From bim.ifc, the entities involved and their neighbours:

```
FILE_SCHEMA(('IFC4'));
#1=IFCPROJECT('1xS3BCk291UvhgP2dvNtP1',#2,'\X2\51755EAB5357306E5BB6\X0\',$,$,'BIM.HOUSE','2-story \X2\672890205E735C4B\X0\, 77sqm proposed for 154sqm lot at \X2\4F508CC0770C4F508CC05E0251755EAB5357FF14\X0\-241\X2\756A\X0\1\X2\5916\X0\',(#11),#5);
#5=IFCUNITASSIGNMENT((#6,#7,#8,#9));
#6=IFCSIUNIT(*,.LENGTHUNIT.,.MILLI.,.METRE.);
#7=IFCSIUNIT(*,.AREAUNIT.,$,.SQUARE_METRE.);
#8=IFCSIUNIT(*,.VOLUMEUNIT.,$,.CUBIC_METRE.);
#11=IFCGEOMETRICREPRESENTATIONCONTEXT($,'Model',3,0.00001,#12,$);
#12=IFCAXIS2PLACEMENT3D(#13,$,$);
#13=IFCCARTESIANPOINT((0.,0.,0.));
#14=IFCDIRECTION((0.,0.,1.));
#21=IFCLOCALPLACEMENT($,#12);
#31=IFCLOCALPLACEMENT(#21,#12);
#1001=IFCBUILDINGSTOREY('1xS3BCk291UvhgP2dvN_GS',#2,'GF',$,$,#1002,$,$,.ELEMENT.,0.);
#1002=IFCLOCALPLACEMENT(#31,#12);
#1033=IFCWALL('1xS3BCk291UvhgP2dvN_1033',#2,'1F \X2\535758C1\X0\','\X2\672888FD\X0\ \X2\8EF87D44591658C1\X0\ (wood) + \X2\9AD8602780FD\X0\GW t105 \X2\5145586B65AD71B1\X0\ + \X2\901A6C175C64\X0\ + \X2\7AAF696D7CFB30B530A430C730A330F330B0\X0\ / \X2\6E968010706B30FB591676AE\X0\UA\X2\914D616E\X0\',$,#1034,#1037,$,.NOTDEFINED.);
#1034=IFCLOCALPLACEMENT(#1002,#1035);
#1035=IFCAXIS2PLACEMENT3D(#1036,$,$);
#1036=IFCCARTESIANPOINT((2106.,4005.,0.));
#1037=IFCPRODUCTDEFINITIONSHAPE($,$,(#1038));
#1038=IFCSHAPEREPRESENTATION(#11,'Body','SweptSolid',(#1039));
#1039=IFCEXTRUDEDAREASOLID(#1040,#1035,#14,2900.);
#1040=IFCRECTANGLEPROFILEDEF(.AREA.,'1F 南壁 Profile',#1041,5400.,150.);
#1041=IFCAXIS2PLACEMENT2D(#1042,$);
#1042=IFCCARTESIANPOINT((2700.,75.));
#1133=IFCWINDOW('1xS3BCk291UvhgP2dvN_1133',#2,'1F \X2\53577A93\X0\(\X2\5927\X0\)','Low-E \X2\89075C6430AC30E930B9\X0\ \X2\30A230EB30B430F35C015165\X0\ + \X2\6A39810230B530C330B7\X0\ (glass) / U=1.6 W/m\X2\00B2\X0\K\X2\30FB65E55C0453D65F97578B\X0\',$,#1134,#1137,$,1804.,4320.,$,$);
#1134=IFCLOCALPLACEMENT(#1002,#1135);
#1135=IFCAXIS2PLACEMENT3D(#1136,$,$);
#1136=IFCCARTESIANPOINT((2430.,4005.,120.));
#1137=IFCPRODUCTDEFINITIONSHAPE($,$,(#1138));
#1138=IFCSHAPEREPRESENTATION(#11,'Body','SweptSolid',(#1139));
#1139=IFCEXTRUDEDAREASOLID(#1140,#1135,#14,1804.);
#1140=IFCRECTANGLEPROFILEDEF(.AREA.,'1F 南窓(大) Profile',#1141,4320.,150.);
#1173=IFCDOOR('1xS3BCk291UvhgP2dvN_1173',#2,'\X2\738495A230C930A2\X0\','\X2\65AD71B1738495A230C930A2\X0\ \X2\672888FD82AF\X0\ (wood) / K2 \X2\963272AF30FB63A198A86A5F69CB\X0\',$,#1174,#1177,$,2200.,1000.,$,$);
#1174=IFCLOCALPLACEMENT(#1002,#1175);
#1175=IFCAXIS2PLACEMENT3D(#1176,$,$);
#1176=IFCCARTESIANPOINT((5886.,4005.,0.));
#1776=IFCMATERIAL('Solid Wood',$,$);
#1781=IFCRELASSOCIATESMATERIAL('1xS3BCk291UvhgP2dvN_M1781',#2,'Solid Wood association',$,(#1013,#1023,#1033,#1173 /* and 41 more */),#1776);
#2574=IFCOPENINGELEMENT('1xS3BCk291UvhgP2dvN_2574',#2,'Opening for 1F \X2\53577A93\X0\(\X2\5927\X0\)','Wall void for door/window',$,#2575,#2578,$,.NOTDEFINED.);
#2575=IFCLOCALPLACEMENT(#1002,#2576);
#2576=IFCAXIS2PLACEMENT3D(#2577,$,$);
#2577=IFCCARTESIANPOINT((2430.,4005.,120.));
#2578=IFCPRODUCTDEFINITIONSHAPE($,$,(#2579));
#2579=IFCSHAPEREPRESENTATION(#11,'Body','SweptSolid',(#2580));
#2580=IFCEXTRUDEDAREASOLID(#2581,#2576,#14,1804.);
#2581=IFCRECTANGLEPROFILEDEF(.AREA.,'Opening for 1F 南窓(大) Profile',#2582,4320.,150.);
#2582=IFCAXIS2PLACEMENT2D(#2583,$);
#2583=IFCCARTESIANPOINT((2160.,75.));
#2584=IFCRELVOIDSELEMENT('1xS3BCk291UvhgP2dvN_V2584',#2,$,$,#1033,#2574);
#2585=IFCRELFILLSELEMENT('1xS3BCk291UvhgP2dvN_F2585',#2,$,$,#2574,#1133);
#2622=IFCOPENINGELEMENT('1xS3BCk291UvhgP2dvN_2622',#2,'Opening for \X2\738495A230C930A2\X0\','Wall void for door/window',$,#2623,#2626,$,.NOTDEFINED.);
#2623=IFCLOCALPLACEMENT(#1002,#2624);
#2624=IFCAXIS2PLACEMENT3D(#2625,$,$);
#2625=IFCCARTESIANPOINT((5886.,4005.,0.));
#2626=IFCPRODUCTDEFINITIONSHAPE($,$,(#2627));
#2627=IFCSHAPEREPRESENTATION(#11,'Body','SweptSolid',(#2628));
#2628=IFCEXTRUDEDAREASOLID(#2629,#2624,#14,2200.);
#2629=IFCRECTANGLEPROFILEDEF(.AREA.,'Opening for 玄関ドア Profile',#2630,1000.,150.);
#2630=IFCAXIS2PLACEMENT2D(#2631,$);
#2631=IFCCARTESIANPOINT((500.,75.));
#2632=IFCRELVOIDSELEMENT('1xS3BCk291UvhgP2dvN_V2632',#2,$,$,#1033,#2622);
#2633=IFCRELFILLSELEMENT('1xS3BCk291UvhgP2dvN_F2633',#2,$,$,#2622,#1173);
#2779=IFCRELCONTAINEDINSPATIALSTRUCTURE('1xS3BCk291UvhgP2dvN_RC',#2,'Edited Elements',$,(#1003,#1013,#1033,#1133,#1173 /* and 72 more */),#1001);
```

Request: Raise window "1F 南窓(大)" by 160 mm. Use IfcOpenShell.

```python
import numpy as np
import ifcopenshell
import ifcopenshell.api.geometry
import ifcopenshell.util.placement
import ifcopenshell.util.unit

model = ifcopenshell.open("bim.ifc")
unit_scale = ifcopenshell.util.unit.calculate_unit_scale(model)

window = model.by_guid("1xS3BCk291UvhgP2dvN_1133")
opening = window.FillsVoids[0].RelatingOpeningElement
dz = 0.16 / unit_scale

shift = np.array([0.0, 0.0, dz])
# The window is not placed relative to its opening, so move both.
for product in (opening, window):
    matrix = ifcopenshell.util.placement.get_local_placement(product.ObjectPlacement)
    matrix[:3, 3] += shift
    ifcopenshell.api.geometry.edit_object_placement(model, product=product, matrix=matrix, is_si=False)

print(f"moved by {dz * unit_scale:+.3f} m")

model.write("bim_v2.ifc")
```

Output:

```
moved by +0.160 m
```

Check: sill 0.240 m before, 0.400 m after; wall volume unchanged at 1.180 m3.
